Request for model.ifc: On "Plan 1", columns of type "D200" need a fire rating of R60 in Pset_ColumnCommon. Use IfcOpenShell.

First a look at what the model holds.

```python
import ifcopenshell
import ifcopenshell.util.element

model = ifcopenshell.open("model.ifc")
print(model.schema)
storey = next(s for s in model.by_type("IfcBuildingStorey") if s.Name == "Plan 1")
columns = [e for e in ifcopenshell.util.element.get_decomposition(storey) if e.is_a("IfcColumn")]
seen = {}
for e in columns:
    element_type = ifcopenshell.util.element.get_type(e)
    key = (element_type.Name if element_type != e and element_type else None, ifcopenshell.util.element.get_pset(e, "Pset_ColumnCommon", "FireRating"))
    seen[key] = seen.get(key, 0) + 1
for (name, value), count in sorted(seen.items(), key=str):
    print(count, "x", name, "|", value)
```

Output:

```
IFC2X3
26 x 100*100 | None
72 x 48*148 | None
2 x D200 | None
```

```python
import ifcopenshell
import ifcopenshell.api.pset
import ifcopenshell.util.element

model = ifcopenshell.open("model.ifc")

storey = next(s for s in model.by_type("IfcBuildingStorey") if s.Name == "Plan 1")
columns = [e for e in ifcopenshell.util.element.get_decomposition(storey) if e.is_a("IfcColumn")]

count = 0
for e in columns:
    element_type = ifcopenshell.util.element.get_type(e)
    if element_type in (None, e) or element_type.Name != "D200":
        continue
    found = ifcopenshell.util.element.get_pset(e, "Pset_ColumnCommon", should_inherit=False)
    if found:
        pset = model.by_id(found["id"])
        if len(ifcopenshell.util.element.get_elements_by_pset(pset)) > 1:
            pset = ifcopenshell.api.pset.unshare_pset(model, products=[e], pset=pset)[0]
    else:
        pset = ifcopenshell.api.pset.add_pset(model, product=e, name="Pset_ColumnCommon")
    ifcopenshell.api.pset.edit_pset(model, pset=pset, properties={"FireRating": "R60"})
    count += 1

print(count, "columns updated")

model.write("model_rev.ifc")
```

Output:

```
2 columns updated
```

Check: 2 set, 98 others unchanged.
